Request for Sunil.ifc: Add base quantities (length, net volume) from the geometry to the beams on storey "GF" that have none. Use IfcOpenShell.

First a look at what the model holds.

```python
import ifcopenshell
import ifcopenshell.util.element
import ifcopenshell.util.unit

model = ifcopenshell.open("Sunil.ifc")
print(model.schema)
for unit_type in ("LENGTHUNIT", "AREAUNIT", "VOLUMEUNIT"):
    print(unit_type, ifcopenshell.util.unit.calculate_unit_scale(model, unit_type))
storey = next(s for s in model.by_type("IfcBuildingStorey") if s.Name == "GF")
beams = [e for e in ifcopenshell.util.element.get_decomposition(storey) if e.is_a("IfcBeam")]
for e in sorted(beams, key=lambda e: e.id()):
    print(e.id(), e.is_a(), e.Name, list(ifcopenshell.util.element.get_psets(e, qtos_only=True)), sep=" | ")
```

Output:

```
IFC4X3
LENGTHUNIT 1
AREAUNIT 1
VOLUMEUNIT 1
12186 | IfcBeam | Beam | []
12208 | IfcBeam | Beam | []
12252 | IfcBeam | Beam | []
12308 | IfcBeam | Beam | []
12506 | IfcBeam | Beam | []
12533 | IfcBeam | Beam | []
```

```python
import ifcopenshell
import ifcopenshell.api.pset
import ifcopenshell.geom
import ifcopenshell.util.element
import ifcopenshell.util.shape
import ifcopenshell.util.unit

model = ifcopenshell.open("Sunil.ifc")
unit_scale = ifcopenshell.util.unit.calculate_unit_scale(model)
volume_scale = ifcopenshell.util.unit.calculate_unit_scale(model, "VOLUMEUNIT")
settings = ifcopenshell.geom.settings()

storey = next(s for s in model.by_type("IfcBuildingStorey") if s.Name == "GF")
beams = [e for e in ifcopenshell.util.element.get_decomposition(storey) if e.is_a("IfcBeam")]

for e in sorted(beams, key=lambda e: e.id()):
    if ifcopenshell.util.element.get_psets(e, qtos_only=True, should_inherit=False):
        continue
    # Geometry comes back in metres, in the element's own axes.
    shape = ifcopenshell.geom.create_shape(settings, e)
    values = {
        "Length": ifcopenshell.util.shape.get_max_xyz(shape.geometry) / unit_scale,
        "NetVolume": ifcopenshell.util.shape.get_volume(shape.geometry) / volume_scale,
    }
    qto = ifcopenshell.api.pset.add_qto(model, product=e, name="Qto_BeamBaseQuantities")
    ifcopenshell.api.pset.edit_qto(model, qto=qto, properties=values)
    print(e.id(), {k: round(v, 3) for k, v in values.items()})

model.write("Sunil_edited.ifc")
```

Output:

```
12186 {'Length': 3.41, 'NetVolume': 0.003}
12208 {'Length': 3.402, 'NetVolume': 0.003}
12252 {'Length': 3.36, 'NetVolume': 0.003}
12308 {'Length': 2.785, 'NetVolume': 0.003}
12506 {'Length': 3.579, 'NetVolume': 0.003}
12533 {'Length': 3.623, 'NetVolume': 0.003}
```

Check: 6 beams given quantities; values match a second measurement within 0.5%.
